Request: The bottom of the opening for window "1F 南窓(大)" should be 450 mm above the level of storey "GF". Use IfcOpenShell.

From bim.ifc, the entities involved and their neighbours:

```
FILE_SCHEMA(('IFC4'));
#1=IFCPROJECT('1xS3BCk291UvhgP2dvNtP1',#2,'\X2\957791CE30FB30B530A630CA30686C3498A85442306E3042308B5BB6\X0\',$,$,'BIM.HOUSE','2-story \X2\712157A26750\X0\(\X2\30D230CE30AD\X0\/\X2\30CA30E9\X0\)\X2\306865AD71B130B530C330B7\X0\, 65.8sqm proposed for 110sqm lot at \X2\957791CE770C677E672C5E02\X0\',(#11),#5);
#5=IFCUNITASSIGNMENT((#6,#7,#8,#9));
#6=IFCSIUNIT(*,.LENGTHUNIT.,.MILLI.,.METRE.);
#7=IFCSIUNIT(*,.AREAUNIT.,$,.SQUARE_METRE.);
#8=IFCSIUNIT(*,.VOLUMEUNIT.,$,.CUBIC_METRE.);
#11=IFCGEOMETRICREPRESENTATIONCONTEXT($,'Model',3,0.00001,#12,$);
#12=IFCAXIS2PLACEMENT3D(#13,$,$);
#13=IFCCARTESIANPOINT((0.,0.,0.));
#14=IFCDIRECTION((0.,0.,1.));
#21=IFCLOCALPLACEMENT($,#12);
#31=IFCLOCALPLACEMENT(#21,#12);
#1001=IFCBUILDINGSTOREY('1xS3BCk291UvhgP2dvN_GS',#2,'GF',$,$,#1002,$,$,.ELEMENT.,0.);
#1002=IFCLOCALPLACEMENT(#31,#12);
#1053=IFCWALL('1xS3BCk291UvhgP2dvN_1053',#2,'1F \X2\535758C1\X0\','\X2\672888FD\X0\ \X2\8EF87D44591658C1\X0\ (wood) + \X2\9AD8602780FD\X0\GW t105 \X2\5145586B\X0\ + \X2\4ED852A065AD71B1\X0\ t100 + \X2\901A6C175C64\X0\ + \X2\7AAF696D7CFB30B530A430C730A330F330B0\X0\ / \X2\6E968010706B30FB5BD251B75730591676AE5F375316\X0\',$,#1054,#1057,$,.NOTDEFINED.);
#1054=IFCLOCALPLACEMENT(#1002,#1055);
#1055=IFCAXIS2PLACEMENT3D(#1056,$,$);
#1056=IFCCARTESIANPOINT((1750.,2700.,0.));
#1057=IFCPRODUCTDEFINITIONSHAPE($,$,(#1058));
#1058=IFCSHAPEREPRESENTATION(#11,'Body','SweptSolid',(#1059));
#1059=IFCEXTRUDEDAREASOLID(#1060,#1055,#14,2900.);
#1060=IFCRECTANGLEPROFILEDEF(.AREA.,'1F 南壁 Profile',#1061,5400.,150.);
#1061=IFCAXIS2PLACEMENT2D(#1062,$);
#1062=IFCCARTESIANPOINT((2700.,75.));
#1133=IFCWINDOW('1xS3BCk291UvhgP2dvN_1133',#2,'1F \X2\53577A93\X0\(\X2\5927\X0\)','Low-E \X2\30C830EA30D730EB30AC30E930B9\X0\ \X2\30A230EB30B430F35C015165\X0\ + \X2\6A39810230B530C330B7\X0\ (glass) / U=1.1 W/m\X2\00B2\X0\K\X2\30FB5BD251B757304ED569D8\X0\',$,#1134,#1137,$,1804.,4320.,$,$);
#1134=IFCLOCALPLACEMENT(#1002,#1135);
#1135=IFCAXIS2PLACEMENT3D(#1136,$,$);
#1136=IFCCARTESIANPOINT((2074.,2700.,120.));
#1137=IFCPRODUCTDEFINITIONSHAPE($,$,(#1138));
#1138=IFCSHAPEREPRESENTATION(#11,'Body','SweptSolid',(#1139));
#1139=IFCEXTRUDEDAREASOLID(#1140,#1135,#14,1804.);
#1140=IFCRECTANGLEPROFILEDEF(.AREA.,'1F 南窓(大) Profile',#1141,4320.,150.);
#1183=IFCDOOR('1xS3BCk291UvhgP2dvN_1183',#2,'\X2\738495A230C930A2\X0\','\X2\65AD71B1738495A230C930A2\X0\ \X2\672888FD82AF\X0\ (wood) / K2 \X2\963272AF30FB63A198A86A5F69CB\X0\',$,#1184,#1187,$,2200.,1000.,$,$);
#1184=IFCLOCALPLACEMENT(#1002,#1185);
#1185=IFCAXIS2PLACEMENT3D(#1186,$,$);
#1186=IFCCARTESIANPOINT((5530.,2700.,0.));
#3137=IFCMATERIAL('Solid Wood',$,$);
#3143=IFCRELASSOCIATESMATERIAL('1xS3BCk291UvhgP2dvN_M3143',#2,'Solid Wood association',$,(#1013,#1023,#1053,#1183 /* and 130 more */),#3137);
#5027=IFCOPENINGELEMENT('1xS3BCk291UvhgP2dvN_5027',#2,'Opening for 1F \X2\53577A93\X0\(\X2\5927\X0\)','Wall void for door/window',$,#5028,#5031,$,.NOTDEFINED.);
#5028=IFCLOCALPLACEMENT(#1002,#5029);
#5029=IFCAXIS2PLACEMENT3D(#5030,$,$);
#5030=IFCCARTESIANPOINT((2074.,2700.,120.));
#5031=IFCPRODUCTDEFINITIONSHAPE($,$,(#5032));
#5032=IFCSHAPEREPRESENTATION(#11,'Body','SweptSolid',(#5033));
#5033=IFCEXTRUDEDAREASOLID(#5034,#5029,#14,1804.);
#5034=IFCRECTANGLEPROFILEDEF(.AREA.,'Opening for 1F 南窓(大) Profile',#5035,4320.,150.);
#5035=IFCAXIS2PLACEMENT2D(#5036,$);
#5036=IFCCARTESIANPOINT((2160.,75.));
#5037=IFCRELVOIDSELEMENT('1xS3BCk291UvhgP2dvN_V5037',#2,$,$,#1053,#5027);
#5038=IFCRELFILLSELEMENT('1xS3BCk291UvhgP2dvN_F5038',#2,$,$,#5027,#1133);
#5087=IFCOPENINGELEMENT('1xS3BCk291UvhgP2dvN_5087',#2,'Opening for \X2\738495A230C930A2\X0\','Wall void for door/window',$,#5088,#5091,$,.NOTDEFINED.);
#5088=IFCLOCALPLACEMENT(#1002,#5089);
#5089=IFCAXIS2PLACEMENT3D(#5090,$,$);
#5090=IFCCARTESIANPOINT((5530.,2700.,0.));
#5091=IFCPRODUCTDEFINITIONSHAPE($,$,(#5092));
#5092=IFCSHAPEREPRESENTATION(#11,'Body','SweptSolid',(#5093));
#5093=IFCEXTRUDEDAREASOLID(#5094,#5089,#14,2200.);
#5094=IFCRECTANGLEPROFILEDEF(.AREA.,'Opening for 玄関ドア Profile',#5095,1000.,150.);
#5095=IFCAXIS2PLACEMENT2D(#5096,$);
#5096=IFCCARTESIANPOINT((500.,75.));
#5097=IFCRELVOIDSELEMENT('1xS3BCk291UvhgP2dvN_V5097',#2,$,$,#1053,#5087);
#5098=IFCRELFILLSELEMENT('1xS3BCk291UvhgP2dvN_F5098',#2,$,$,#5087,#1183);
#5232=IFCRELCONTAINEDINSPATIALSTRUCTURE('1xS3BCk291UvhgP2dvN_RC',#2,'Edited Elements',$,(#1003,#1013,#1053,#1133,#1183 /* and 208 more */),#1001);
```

```python
import numpy as np
import ifcopenshell
import ifcopenshell.api.geometry
import ifcopenshell.geom
import ifcopenshell.util.element
import ifcopenshell.util.placement
import ifcopenshell.util.shape
import ifcopenshell.util.unit

model = ifcopenshell.open("bim.ifc")
unit_scale = ifcopenshell.util.unit.calculate_unit_scale(model)

window = model.by_guid("1xS3BCk291UvhgP2dvN_1133")
opening = window.FillsVoids[0].RelatingOpeningElement
storey = ifcopenshell.util.element.get_container(window, ifc_class="IfcBuildingStorey")
level = ifcopenshell.util.placement.get_local_placement(storey.ObjectPlacement)[2, 3]

# The opening's origin need not be at the sill, so measure its lowest point.
shape = ifcopenshell.geom.create_shape(ifcopenshell.geom.settings(), opening)
bottom = ifcopenshell.util.shape.get_shape_bottom_elevation(shape, shape.geometry) / unit_scale
dz = level + 0.45 / unit_scale - bottom

shift = np.array([0.0, 0.0, dz])
# The window is not placed relative to its opening, so move both.
for product in (opening, window):
    matrix = ifcopenshell.util.placement.get_local_placement(product.ObjectPlacement)
    matrix[:3, 3] += shift
    ifcopenshell.api.geometry.edit_object_placement(model, product=product, matrix=matrix, is_si=False)

print(f"moved by {dz * unit_scale:+.3f} m")

model.write("bim_rev.ifc")
```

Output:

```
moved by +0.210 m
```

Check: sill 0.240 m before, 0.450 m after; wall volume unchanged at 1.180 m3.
